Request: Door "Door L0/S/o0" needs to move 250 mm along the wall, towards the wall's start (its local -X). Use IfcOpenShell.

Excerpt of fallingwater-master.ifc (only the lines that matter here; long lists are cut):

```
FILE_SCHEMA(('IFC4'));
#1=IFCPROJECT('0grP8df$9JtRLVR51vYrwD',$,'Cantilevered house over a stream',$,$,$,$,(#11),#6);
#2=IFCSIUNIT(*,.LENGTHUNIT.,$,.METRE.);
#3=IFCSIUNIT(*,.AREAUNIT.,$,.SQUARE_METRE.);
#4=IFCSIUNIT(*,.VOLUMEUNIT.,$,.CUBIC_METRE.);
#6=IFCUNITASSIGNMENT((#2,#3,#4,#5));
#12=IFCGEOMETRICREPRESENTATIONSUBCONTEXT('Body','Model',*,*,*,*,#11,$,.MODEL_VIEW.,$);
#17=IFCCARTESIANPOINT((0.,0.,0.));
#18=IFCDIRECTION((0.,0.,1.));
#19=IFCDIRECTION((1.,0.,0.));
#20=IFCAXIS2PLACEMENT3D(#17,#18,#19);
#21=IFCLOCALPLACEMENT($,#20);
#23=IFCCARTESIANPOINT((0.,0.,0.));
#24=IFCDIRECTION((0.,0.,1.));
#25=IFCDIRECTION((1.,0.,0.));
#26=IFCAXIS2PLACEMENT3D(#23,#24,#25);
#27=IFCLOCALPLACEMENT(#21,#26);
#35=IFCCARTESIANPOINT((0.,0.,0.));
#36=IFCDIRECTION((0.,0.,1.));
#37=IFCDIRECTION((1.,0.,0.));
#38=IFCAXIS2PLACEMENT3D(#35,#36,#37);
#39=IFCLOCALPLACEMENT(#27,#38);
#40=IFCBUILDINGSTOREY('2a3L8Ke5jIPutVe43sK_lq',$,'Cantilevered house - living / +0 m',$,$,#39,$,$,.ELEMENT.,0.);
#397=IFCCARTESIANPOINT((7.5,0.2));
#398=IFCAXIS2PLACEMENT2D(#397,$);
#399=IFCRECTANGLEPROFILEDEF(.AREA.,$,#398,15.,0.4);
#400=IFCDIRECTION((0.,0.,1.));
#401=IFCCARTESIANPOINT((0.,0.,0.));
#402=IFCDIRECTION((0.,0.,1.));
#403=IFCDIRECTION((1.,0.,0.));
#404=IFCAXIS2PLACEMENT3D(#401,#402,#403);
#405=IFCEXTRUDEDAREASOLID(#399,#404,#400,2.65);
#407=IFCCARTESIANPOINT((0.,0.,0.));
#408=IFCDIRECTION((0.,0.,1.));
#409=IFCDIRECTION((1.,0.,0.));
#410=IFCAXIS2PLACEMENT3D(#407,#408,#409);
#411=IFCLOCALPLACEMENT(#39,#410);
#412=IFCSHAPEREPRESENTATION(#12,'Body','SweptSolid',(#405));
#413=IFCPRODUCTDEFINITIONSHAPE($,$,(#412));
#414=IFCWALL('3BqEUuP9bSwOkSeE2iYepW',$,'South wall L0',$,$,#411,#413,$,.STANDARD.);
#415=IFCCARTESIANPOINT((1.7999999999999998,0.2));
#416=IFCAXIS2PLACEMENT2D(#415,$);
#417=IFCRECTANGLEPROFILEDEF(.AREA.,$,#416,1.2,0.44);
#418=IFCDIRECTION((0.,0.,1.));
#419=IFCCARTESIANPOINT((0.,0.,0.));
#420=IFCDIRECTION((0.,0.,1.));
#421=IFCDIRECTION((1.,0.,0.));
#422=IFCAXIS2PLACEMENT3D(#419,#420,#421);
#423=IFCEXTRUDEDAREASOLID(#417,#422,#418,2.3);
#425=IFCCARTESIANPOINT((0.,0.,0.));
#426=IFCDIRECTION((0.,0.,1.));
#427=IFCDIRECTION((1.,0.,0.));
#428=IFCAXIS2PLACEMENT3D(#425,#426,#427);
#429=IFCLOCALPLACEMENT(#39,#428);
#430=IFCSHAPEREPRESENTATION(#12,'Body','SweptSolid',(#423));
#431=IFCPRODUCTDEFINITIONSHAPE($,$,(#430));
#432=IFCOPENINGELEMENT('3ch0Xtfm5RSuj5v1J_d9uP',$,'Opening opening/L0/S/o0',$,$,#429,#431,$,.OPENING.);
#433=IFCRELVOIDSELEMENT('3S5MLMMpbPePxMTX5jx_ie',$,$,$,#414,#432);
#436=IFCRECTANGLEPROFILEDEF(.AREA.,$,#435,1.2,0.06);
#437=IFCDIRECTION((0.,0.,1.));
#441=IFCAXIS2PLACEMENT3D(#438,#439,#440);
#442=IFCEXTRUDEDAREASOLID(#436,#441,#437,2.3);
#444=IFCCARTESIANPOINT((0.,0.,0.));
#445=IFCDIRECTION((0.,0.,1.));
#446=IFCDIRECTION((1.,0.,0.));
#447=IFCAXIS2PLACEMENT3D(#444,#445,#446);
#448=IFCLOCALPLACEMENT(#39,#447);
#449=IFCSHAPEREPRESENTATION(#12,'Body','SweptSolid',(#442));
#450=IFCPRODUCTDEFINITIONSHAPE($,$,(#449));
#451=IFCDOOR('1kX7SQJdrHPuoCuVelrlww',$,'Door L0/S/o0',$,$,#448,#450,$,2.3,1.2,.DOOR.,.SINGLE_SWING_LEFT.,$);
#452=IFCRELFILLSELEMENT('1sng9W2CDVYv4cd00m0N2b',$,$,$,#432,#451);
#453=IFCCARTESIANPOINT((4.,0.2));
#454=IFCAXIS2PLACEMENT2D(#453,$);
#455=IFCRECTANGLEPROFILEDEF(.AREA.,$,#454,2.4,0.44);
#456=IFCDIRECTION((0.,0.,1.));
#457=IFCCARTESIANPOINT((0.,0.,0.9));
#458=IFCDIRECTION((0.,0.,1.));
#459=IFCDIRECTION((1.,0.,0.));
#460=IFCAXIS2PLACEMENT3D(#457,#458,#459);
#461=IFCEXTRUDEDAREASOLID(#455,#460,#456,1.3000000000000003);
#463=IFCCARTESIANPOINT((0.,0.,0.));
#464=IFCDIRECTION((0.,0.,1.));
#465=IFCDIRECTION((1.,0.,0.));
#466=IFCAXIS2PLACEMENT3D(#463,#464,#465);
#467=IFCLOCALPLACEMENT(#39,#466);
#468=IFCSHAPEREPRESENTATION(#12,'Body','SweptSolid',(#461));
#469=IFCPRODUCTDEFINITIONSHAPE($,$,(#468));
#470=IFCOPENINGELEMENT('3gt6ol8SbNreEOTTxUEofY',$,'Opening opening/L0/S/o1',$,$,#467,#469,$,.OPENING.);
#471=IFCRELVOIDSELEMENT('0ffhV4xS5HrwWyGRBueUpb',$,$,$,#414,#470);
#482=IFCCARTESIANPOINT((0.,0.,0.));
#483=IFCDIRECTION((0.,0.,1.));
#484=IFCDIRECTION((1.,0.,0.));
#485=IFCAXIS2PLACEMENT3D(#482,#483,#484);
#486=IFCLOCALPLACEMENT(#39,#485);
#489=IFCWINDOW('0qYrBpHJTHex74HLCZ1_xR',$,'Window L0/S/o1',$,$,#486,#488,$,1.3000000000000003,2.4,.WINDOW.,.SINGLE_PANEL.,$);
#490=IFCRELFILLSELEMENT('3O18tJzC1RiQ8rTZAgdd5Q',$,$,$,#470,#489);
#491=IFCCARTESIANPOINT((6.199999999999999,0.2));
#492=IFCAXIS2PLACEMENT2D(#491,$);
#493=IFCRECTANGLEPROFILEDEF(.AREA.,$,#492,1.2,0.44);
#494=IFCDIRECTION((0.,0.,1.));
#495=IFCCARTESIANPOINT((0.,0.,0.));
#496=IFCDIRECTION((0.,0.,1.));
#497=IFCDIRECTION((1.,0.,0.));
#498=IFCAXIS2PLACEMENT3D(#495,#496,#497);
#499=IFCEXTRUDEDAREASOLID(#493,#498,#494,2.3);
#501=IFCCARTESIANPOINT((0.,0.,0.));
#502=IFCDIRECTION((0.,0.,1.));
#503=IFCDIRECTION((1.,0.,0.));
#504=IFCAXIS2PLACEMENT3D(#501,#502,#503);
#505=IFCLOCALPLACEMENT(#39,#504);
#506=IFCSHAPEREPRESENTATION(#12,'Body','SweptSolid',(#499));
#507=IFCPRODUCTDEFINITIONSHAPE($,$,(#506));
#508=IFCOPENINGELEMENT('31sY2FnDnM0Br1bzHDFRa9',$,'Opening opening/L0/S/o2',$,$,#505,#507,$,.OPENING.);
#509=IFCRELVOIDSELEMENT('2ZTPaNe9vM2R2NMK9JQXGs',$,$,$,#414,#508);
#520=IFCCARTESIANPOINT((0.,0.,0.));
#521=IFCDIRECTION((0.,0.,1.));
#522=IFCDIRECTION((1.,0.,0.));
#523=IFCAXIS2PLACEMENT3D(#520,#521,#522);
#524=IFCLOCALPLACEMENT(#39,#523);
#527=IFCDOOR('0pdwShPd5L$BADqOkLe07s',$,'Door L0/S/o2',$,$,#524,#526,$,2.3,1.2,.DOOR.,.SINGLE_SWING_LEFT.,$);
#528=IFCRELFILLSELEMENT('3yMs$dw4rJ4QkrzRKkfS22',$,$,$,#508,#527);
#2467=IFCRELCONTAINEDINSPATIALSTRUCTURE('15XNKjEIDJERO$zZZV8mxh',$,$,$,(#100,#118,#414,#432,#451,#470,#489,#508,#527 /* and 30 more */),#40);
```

```python
import ifcopenshell
import ifcopenshell.api.geometry
import ifcopenshell.util.placement
import ifcopenshell.util.unit

model = ifcopenshell.open("fallingwater-master.ifc")
unit_scale = ifcopenshell.util.unit.calculate_unit_scale(model)

door = model.by_id(451)
opening = door.FillsVoids[0].RelatingOpeningElement
wall = opening.VoidsElements[0].RelatingBuildingElement

wall_matrix = ifcopenshell.util.placement.get_local_placement(wall.ObjectPlacement)
shift = wall_matrix[:3, 0] * -0.25 / unit_scale
before = ifcopenshell.util.placement.get_local_placement(door.ObjectPlacement)[:3, 3].copy()

# The door is not placed relative to its opening, so move both.
for product in (opening, door):
    matrix = ifcopenshell.util.placement.get_local_placement(product.ObjectPlacement)
    matrix[:3, 3] += shift
    ifcopenshell.api.geometry.edit_object_placement(model, product=product, matrix=matrix, is_si=False)

after = ifcopenshell.util.placement.get_local_placement(door.ObjectPlacement)[:3, 3]
print("door moved by", (after - before).round(3) + 0.0)

model.write("fallingwater-master_rev.ifc")
```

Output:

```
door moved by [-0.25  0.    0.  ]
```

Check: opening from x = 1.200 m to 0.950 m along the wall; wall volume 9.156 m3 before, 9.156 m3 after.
